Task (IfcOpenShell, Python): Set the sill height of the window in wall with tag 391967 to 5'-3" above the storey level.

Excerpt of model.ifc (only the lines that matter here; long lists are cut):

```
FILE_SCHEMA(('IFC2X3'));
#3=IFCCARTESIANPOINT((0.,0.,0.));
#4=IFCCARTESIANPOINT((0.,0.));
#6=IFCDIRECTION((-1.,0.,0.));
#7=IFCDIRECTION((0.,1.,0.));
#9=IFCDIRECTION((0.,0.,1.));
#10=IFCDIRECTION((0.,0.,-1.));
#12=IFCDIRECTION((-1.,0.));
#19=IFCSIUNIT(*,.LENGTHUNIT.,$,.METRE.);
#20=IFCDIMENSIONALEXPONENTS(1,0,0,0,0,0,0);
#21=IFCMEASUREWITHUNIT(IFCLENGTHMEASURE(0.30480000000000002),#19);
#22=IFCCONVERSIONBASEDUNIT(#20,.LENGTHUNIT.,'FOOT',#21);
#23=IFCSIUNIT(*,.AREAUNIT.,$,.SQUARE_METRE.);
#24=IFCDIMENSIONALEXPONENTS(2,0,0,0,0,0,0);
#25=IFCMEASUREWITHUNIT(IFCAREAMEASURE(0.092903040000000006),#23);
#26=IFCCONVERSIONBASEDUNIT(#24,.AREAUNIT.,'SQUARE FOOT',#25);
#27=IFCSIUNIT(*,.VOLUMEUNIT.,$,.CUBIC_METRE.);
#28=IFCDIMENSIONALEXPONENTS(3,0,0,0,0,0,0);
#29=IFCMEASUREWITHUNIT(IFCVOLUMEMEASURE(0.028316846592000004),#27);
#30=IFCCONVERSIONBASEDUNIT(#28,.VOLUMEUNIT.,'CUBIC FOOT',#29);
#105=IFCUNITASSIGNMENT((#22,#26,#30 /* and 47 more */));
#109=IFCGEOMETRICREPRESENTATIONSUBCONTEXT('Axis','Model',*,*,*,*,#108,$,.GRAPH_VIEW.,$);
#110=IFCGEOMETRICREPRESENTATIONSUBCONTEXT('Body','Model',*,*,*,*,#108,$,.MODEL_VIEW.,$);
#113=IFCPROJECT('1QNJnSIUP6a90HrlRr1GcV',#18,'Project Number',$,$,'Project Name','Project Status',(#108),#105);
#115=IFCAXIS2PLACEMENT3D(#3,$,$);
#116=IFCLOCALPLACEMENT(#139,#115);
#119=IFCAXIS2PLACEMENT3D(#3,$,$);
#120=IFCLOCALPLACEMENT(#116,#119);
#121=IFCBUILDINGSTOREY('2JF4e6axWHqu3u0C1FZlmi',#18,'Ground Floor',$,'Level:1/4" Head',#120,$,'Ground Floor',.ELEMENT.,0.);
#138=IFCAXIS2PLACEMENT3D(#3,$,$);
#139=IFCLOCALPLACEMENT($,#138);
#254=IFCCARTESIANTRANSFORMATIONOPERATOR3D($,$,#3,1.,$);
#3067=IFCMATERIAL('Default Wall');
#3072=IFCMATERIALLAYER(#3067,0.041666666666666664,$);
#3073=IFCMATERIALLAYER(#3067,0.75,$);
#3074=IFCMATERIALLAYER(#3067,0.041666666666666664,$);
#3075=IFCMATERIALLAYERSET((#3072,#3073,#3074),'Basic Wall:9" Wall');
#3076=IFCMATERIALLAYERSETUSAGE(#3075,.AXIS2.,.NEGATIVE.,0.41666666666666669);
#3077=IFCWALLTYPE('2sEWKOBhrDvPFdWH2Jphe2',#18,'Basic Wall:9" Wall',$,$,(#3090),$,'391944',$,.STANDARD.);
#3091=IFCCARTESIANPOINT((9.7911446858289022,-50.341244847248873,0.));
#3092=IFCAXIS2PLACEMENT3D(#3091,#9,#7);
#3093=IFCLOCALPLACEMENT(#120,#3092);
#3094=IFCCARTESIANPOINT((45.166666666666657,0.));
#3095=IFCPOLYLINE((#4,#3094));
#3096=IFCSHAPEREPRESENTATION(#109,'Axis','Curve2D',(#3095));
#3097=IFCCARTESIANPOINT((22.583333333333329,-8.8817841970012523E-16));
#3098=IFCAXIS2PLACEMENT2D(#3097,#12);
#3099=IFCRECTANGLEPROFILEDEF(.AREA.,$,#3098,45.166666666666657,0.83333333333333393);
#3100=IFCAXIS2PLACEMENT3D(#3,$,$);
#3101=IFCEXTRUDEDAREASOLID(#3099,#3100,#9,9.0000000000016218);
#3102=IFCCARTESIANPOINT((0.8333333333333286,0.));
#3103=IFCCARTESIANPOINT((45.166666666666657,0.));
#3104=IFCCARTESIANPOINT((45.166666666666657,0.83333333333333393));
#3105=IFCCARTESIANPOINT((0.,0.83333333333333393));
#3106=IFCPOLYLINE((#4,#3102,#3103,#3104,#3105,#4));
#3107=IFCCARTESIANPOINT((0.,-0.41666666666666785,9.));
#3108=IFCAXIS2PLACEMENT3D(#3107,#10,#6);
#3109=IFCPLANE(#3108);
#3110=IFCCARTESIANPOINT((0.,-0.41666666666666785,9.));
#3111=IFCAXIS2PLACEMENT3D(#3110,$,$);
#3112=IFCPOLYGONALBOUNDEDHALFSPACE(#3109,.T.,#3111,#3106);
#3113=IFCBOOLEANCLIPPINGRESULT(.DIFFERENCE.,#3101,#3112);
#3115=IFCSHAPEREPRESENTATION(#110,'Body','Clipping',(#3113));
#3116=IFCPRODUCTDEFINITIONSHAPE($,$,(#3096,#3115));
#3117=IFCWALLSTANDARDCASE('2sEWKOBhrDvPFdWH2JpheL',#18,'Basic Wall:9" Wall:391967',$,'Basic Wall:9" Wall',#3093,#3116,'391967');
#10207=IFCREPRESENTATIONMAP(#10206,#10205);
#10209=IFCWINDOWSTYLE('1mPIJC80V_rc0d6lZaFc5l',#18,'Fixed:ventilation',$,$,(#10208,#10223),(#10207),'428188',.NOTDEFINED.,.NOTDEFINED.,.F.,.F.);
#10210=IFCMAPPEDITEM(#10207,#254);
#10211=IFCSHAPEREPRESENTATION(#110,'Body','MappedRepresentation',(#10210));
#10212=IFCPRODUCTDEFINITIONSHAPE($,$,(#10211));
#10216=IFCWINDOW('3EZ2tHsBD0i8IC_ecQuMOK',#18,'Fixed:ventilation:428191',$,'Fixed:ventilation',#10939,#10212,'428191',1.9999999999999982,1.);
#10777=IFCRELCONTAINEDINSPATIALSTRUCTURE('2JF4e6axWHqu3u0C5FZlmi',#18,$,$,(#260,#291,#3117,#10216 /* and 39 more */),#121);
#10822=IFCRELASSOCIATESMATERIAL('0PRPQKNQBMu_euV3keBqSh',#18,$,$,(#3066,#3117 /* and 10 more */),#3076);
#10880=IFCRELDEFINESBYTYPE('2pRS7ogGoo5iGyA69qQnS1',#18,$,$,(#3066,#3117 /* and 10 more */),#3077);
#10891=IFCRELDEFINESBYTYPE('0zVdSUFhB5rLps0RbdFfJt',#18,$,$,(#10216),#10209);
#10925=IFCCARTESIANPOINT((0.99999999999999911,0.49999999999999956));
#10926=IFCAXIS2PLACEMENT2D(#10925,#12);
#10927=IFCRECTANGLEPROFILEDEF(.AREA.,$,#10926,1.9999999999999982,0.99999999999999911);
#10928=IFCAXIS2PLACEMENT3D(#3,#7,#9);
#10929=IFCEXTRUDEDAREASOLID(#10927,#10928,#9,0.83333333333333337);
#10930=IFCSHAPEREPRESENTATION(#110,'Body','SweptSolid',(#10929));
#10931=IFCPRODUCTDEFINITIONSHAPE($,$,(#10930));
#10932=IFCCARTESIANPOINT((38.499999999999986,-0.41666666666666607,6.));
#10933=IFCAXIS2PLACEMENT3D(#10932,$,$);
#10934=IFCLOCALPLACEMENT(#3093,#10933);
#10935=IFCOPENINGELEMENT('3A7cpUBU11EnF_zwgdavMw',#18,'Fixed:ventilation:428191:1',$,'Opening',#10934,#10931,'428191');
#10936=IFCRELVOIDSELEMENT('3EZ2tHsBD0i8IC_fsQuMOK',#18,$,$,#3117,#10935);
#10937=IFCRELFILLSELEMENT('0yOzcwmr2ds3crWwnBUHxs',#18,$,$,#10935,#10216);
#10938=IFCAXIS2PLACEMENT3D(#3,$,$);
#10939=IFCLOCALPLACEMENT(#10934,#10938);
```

```python
import numpy as np
import ifcopenshell
import ifcopenshell.api.geometry
import ifcopenshell.geom
import ifcopenshell.util.element
import ifcopenshell.util.placement
import ifcopenshell.util.shape
import ifcopenshell.util.unit

model = ifcopenshell.open("model.ifc")
unit_scale = ifcopenshell.util.unit.calculate_unit_scale(model)

window = model.by_guid("3EZ2tHsBD0i8IC_ecQuMOK")
opening = window.FillsVoids[0].RelatingOpeningElement
storey = ifcopenshell.util.element.get_container(window, ifc_class="IfcBuildingStorey")
level = ifcopenshell.util.placement.get_local_placement(storey.ObjectPlacement)[2, 3]

# The opening's origin need not be at the sill, so measure its lowest point.
shape = ifcopenshell.geom.create_shape(ifcopenshell.geom.settings(), opening)
bottom = ifcopenshell.util.shape.get_shape_bottom_elevation(shape, shape.geometry) / unit_scale
dz = level + 63 * 0.0254 / unit_scale - bottom

shift = np.array([0.0, 0.0, dz])
# The window is placed relative to its opening, so it follows when the opening moves.
matrix = ifcopenshell.util.placement.get_local_placement(opening.ObjectPlacement)
matrix[:3, 3] += shift
ifcopenshell.api.geometry.edit_object_placement(
    model, product=opening, matrix=matrix, is_si=False, should_transform_children=True
)

print(f"moved by {dz * unit_scale:+.3f} m")

model.write("model_updated.ifc")
```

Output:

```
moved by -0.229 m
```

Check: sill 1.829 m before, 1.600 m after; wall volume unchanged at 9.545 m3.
